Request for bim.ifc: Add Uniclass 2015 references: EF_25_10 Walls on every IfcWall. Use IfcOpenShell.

First a look at what the model holds.

```python
import ifcopenshell

model = ifcopenshell.open("bim.ifc")
print(model.schema)
print("classifications:", [c.Name for c in model.by_type("IfcClassification")])
for ifc_class in ("IfcDoor", "IfcRoof", "IfcStair", "IfcWall", "IfcWindow"):
    print(ifc_class, len(model.by_type(ifc_class)))
```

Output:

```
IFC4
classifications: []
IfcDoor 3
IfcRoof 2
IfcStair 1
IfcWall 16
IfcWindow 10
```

```python
import ifcopenshell
import ifcopenshell.api.classification

model = ifcopenshell.open("bim.ifc")

system = ifcopenshell.api.classification.add_classification(model, classification="Uniclass 2015")

codes = {
    "IfcWall": ("EF_25_10", "Walls"),
}
for ifc_class, (code, name) in codes.items():
    products = model.by_type(ifc_class)
    ifcopenshell.api.classification.add_reference(
        model, products=products, classification=system, identification=code, name=name
    )
    print(code, len(products))

model.write("bim_v2.ifc")
```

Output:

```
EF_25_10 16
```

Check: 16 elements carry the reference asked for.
